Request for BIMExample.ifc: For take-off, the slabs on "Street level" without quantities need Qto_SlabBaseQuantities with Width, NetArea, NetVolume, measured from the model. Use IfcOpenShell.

First a look at what the model holds.

```python
import ifcopenshell
import ifcopenshell.util.element
import ifcopenshell.util.unit

model = ifcopenshell.open("BIMExample.ifc")
print(model.schema)
for unit_type in ("LENGTHUNIT", "AREAUNIT", "VOLUMEUNIT"):
    print(unit_type, ifcopenshell.util.unit.calculate_unit_scale(model, unit_type))
storey = next(s for s in model.by_type("IfcBuildingStorey") if s.Name == "Street level")
slabs = [e for e in ifcopenshell.util.element.get_decomposition(storey) if e.is_a("IfcSlab")]
for e in sorted(slabs, key=lambda e: e.id()):
    print(e.id(), e.is_a(), e.Name, list(ifcopenshell.util.element.get_psets(e, qtos_only=True)), sep=" | ")
```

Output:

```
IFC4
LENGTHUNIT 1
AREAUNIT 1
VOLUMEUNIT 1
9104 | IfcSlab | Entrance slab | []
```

```python
import ifcopenshell
import ifcopenshell.api.pset
import ifcopenshell.geom
import ifcopenshell.util.element
import ifcopenshell.util.shape
import ifcopenshell.util.unit

model = ifcopenshell.open("BIMExample.ifc")
unit_scale = ifcopenshell.util.unit.calculate_unit_scale(model)
area_scale = ifcopenshell.util.unit.calculate_unit_scale(model, "AREAUNIT")
volume_scale = ifcopenshell.util.unit.calculate_unit_scale(model, "VOLUMEUNIT")
settings = ifcopenshell.geom.settings()

storey = next(s for s in model.by_type("IfcBuildingStorey") if s.Name == "Street level")
slabs = [e for e in ifcopenshell.util.element.get_decomposition(storey) if e.is_a("IfcSlab")]

for e in sorted(slabs, key=lambda e: e.id()):
    if ifcopenshell.util.element.get_psets(e, qtos_only=True, should_inherit=False):
        continue
    # Geometry comes back in metres, in the element's own axes.
    shape = ifcopenshell.geom.create_shape(settings, e)
    values = {
        "Width": ifcopenshell.util.shape.get_z(shape.geometry) / unit_scale,
        "NetArea": ifcopenshell.util.shape.get_footprint_area(shape.geometry) / area_scale,
        "NetVolume": ifcopenshell.util.shape.get_volume(shape.geometry) / volume_scale,
    }
    qto = ifcopenshell.api.pset.add_qto(model, product=e, name="Qto_SlabBaseQuantities")
    ifcopenshell.api.pset.edit_qto(model, qto=qto, properties=values)
    print(e.id(), {k: round(v, 3) for k, v in values.items()})

model.write("BIMExample_v2.ifc")
```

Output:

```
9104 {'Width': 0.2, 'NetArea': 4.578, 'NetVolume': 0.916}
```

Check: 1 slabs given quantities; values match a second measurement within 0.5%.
